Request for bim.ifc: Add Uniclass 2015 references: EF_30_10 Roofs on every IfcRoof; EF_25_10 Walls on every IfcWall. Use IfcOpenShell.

First a look at what the model holds.

```python
import ifcopenshell

model = ifcopenshell.open("bim.ifc")
print(model.schema)
print("classifications:", [c.Name for c in model.by_type("IfcClassification")])
for ifc_class in ("IfcDoor", "IfcRoof", "IfcStair", "IfcWall", "IfcWindow"):
    print(ifc_class, len(model.by_type(ifc_class)))
```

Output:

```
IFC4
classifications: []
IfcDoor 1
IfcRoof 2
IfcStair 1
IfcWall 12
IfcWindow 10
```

```python
import ifcopenshell
import ifcopenshell.api.classification

model = ifcopenshell.open("bim.ifc")

system = ifcopenshell.api.classification.add_classification(model, classification="Uniclass 2015")

codes = {
    "IfcRoof": ("EF_30_10", "Roofs"),
    "IfcWall": ("EF_25_10", "Walls"),
}
for ifc_class, (code, name) in codes.items():
    products = model.by_type(ifc_class)
    ifcopenshell.api.classification.add_reference(
        model, products=products, classification=system, identification=code, name=name
    )
    print(code, len(products))

model.write("bim_updated.ifc")
```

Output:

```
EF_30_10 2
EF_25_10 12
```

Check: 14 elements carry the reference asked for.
